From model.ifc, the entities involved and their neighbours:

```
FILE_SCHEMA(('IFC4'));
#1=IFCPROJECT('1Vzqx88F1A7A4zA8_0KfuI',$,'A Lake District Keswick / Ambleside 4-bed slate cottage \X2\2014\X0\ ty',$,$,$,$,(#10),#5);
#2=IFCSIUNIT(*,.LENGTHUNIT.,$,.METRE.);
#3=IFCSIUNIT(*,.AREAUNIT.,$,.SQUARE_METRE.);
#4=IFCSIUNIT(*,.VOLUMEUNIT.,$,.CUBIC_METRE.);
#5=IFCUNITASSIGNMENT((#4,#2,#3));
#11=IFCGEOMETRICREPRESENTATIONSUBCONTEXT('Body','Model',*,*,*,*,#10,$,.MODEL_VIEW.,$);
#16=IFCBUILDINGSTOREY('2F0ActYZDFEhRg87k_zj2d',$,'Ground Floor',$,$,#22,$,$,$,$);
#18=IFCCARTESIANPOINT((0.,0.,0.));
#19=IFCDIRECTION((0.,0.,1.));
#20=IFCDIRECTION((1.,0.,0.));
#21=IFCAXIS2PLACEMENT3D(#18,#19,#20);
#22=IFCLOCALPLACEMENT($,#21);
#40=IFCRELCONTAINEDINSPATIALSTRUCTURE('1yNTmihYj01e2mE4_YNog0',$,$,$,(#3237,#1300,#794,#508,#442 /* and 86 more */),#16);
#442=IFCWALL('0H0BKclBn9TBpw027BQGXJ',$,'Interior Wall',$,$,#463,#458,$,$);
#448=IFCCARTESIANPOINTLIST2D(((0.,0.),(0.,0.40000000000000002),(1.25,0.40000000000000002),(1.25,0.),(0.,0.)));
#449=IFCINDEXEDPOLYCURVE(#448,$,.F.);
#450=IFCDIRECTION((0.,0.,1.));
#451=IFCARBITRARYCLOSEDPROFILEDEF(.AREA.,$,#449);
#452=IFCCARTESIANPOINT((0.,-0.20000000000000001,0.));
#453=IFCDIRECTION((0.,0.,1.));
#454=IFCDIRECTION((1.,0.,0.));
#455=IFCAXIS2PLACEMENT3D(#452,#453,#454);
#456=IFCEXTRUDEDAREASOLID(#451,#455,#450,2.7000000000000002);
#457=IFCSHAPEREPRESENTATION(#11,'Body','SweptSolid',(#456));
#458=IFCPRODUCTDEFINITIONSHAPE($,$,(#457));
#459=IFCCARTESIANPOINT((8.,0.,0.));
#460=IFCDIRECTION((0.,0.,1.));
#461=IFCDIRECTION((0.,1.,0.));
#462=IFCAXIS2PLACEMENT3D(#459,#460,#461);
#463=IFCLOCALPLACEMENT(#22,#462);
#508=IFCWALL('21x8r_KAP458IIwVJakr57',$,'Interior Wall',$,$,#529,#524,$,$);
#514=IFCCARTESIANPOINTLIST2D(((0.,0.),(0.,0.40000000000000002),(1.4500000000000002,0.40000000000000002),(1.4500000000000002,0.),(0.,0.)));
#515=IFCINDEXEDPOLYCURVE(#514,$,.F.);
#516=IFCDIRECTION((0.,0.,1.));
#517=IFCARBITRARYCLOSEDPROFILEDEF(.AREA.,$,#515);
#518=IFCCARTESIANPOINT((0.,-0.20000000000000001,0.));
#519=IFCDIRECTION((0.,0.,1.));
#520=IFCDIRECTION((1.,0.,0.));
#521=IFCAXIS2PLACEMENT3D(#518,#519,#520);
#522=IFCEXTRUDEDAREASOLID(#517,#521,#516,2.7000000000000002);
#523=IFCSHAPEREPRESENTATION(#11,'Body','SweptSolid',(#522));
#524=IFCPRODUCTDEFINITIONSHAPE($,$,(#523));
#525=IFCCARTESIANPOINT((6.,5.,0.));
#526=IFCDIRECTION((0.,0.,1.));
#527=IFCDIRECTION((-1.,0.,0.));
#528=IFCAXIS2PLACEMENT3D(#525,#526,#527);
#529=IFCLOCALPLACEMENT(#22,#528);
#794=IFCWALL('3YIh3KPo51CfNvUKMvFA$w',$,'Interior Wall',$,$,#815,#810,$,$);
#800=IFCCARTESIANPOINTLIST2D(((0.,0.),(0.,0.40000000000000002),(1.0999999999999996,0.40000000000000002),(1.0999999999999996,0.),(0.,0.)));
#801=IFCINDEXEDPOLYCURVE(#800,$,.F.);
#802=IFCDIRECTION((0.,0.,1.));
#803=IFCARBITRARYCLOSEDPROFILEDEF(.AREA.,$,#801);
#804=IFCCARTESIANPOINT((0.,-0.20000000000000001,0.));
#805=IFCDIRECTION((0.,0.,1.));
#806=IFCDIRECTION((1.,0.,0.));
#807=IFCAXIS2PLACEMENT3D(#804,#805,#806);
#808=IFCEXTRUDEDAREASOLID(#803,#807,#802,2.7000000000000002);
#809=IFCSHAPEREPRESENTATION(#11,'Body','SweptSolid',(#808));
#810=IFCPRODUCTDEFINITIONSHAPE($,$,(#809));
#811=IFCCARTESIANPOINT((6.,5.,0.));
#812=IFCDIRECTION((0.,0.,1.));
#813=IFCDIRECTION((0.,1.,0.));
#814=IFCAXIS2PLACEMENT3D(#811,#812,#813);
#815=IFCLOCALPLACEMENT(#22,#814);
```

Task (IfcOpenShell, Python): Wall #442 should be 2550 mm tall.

```python
import ifcopenshell
import ifcopenshell.geom
import ifcopenshell.util.representation
import ifcopenshell.util.shape
import ifcopenshell.util.unit

model = ifcopenshell.open("model.ifc")
unit_scale = ifcopenshell.util.unit.calculate_unit_scale(model)
settings = ifcopenshell.geom.settings()


def volume(element):
    """Net volume in cubic metres, openings subtracted."""
    shape = ifcopenshell.geom.create_shape(settings, element)
    return ifcopenshell.util.shape.get_volume(shape.geometry)


wall = model.by_guid("0H0BKclBn9TBpw027BQGXJ")
before = volume(wall)

body = ifcopenshell.util.representation.get_representation(wall, "Model", "Body")
solid = body.Items[0]
old_height = solid.Depth
solid.Depth = 2.55 / unit_scale
after = volume(wall)

print(f"height {old_height:g} -> {solid.Depth:g}, volume {before:.3f} -> {after:.3f} m3")

model.write("model-out.ifc")
```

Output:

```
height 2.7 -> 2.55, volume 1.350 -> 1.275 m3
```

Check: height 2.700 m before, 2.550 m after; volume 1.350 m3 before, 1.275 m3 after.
